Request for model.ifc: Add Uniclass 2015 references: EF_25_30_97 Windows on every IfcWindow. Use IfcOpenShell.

First a look at what the model holds.

```python
import ifcopenshell

model = ifcopenshell.open("model.ifc")
print(model.schema)
print("classifications:", [c.Name for c in model.by_type("IfcClassification")])
for ifc_class in ("IfcDoor", "IfcRoof", "IfcStair", "IfcWall", "IfcWindow"):
    print(ifc_class, len(model.by_type(ifc_class)))
```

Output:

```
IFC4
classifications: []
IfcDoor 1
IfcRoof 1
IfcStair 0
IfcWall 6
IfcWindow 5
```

```python
import ifcopenshell
import ifcopenshell.api.classification

model = ifcopenshell.open("model.ifc")

system = ifcopenshell.api.classification.add_classification(model, classification="Uniclass 2015")

codes = {
    "IfcWindow": ("EF_25_30_97", "Windows"),
}
for ifc_class, (code, name) in codes.items():
    products = model.by_type(ifc_class)
    ifcopenshell.api.classification.add_reference(
        model, products=products, classification=system, identification=code, name=name
    )
    print(code, len(products))

model.write("model_rev.ifc")
```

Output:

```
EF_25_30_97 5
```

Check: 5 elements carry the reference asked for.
